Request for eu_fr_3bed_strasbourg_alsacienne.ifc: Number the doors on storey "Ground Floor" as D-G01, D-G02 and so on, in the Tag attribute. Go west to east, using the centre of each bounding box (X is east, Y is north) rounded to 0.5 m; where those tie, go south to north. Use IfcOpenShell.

First a look at what the model holds.

```python
import ifcopenshell
import ifcopenshell.util.element
import ifcopenshell.util.placement

model = ifcopenshell.open("eu_fr_3bed_strasbourg_alsacienne.ifc")
print(model.schema)
storey = next(s for s in model.by_type("IfcBuildingStorey") if s.Name == "Ground Floor")
doors = [e for e in ifcopenshell.util.element.get_decomposition(storey) if e.is_a("IfcDoor")]
for e in sorted(doors, key=lambda e: e.id()):
    origin = ifcopenshell.util.placement.get_local_placement(e.ObjectPlacement)[:3, 3]
    print(e.id(), e.Tag, e.Name, origin.round(2) + 0.0, sep=" | ")
```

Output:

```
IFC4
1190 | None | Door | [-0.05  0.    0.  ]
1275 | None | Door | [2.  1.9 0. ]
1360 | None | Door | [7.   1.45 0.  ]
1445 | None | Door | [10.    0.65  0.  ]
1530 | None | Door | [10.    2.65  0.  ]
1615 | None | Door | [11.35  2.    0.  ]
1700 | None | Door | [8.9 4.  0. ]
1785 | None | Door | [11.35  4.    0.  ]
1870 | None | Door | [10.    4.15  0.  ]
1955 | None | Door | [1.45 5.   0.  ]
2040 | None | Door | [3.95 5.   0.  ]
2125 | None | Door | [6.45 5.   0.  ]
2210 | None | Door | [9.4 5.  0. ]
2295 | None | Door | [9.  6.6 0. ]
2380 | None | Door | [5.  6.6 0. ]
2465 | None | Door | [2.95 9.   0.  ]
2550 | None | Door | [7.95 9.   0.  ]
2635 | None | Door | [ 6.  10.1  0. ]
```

```python
import ifcopenshell
import ifcopenshell.geom
import ifcopenshell.util.element
import ifcopenshell.util.shape

model = ifcopenshell.open("eu_fr_3bed_strasbourg_alsacienne.ifc")
settings = ifcopenshell.geom.settings()
settings.set("use-world-coords", True)


def centre(element):
    shape = ifcopenshell.geom.create_shape(settings, element)
    return ifcopenshell.util.shape.get_bbox_centroid(shape.geometry)


storey = next(s for s in model.by_type("IfcBuildingStorey") if s.Name == "Ground Floor")
doors = [e for e in ifcopenshell.util.element.get_decomposition(storey) if e.is_a("IfcDoor")]

# Insertion points can sit at a corner or the storey origin, so sort by the geometry (in metres).
centres = {e: centre(e) for e in doors}
doors.sort(key=lambda e: (round(centres[e][0] / 0.5), centres[e][1]))

for i, e in enumerate(doors, start=1):
    number = f"D-G{i:02d}"
    e.Tag = number
    print(e.id(), number)

model.write("eu_fr_3bed_strasbourg_alsacienne_updated.ifc")
```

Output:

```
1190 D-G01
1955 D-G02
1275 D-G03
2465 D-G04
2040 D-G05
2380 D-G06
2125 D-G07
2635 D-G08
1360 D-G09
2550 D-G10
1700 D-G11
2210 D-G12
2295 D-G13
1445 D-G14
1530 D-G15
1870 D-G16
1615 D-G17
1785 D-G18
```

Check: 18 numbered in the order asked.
